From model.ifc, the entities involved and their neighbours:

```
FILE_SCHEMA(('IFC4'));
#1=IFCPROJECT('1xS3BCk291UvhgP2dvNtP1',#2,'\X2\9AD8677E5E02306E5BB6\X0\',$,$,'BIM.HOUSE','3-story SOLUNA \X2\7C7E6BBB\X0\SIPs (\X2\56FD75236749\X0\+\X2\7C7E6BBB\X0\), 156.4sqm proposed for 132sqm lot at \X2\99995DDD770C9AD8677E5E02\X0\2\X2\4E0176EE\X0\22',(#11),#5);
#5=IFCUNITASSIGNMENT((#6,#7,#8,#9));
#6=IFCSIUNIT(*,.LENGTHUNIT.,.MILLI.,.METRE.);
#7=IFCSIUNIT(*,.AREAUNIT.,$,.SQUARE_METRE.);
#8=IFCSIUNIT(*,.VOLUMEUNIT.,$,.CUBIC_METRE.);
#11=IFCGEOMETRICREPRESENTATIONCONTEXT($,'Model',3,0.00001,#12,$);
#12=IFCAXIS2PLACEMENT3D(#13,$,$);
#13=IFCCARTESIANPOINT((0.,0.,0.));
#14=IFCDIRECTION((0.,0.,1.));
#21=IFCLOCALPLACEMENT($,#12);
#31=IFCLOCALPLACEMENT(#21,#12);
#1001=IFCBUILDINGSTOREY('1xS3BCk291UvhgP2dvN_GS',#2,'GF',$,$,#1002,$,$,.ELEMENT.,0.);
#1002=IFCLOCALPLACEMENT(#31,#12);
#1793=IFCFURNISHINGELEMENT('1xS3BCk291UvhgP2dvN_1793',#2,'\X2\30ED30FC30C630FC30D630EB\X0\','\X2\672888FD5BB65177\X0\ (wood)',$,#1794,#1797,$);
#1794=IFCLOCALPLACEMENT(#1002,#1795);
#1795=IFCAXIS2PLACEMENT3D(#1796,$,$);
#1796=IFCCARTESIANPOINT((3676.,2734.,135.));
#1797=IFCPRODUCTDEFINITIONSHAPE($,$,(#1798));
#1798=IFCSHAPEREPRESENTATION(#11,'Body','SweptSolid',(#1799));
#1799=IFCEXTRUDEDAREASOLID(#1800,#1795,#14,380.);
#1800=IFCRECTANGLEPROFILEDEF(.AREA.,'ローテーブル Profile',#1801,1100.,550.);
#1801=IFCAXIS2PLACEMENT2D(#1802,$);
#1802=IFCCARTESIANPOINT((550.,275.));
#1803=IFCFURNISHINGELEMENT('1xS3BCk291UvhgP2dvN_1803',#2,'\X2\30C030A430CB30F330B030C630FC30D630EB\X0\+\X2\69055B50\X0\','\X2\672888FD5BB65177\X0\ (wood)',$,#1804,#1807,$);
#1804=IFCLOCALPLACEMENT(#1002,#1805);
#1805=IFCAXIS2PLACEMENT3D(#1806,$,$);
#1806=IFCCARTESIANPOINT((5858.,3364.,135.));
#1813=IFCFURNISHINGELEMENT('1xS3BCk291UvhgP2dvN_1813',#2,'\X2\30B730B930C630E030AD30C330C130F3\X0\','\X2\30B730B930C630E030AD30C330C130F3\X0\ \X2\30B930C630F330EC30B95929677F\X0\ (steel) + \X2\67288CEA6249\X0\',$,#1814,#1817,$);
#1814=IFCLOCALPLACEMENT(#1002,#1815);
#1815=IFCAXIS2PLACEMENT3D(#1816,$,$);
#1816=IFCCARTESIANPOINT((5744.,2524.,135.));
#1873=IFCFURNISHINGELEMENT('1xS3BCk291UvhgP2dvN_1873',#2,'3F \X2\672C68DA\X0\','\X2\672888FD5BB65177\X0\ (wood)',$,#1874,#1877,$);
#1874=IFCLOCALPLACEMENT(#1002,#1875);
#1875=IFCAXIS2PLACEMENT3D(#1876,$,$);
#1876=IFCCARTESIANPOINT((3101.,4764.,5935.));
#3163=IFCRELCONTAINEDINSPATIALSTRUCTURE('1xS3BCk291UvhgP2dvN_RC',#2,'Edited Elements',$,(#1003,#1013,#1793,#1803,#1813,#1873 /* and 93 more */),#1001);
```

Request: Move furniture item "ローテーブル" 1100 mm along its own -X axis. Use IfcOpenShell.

```python
import ifcopenshell
import ifcopenshell.api.geometry
import ifcopenshell.util.placement
import ifcopenshell.util.unit

model = ifcopenshell.open("model.ifc")
unit_scale = ifcopenshell.util.unit.calculate_unit_scale(model)

item = model.by_guid("1xS3BCk291UvhgP2dvN_1793")
matrix = ifcopenshell.util.placement.get_local_placement(item.ObjectPlacement)
matrix[:3, 3] -= matrix[:3, 0] * 1.1 / unit_scale
ifcopenshell.api.geometry.edit_object_placement(model, product=item, matrix=matrix, is_si=False)

print(ifcopenshell.util.placement.get_local_placement(item.ObjectPlacement).round(3) + 0.0)

model.write("model_rev.ifc")
```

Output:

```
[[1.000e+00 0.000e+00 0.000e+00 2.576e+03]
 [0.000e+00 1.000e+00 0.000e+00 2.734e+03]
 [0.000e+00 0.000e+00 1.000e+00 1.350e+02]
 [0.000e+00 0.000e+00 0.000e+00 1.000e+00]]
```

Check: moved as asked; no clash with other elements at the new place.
